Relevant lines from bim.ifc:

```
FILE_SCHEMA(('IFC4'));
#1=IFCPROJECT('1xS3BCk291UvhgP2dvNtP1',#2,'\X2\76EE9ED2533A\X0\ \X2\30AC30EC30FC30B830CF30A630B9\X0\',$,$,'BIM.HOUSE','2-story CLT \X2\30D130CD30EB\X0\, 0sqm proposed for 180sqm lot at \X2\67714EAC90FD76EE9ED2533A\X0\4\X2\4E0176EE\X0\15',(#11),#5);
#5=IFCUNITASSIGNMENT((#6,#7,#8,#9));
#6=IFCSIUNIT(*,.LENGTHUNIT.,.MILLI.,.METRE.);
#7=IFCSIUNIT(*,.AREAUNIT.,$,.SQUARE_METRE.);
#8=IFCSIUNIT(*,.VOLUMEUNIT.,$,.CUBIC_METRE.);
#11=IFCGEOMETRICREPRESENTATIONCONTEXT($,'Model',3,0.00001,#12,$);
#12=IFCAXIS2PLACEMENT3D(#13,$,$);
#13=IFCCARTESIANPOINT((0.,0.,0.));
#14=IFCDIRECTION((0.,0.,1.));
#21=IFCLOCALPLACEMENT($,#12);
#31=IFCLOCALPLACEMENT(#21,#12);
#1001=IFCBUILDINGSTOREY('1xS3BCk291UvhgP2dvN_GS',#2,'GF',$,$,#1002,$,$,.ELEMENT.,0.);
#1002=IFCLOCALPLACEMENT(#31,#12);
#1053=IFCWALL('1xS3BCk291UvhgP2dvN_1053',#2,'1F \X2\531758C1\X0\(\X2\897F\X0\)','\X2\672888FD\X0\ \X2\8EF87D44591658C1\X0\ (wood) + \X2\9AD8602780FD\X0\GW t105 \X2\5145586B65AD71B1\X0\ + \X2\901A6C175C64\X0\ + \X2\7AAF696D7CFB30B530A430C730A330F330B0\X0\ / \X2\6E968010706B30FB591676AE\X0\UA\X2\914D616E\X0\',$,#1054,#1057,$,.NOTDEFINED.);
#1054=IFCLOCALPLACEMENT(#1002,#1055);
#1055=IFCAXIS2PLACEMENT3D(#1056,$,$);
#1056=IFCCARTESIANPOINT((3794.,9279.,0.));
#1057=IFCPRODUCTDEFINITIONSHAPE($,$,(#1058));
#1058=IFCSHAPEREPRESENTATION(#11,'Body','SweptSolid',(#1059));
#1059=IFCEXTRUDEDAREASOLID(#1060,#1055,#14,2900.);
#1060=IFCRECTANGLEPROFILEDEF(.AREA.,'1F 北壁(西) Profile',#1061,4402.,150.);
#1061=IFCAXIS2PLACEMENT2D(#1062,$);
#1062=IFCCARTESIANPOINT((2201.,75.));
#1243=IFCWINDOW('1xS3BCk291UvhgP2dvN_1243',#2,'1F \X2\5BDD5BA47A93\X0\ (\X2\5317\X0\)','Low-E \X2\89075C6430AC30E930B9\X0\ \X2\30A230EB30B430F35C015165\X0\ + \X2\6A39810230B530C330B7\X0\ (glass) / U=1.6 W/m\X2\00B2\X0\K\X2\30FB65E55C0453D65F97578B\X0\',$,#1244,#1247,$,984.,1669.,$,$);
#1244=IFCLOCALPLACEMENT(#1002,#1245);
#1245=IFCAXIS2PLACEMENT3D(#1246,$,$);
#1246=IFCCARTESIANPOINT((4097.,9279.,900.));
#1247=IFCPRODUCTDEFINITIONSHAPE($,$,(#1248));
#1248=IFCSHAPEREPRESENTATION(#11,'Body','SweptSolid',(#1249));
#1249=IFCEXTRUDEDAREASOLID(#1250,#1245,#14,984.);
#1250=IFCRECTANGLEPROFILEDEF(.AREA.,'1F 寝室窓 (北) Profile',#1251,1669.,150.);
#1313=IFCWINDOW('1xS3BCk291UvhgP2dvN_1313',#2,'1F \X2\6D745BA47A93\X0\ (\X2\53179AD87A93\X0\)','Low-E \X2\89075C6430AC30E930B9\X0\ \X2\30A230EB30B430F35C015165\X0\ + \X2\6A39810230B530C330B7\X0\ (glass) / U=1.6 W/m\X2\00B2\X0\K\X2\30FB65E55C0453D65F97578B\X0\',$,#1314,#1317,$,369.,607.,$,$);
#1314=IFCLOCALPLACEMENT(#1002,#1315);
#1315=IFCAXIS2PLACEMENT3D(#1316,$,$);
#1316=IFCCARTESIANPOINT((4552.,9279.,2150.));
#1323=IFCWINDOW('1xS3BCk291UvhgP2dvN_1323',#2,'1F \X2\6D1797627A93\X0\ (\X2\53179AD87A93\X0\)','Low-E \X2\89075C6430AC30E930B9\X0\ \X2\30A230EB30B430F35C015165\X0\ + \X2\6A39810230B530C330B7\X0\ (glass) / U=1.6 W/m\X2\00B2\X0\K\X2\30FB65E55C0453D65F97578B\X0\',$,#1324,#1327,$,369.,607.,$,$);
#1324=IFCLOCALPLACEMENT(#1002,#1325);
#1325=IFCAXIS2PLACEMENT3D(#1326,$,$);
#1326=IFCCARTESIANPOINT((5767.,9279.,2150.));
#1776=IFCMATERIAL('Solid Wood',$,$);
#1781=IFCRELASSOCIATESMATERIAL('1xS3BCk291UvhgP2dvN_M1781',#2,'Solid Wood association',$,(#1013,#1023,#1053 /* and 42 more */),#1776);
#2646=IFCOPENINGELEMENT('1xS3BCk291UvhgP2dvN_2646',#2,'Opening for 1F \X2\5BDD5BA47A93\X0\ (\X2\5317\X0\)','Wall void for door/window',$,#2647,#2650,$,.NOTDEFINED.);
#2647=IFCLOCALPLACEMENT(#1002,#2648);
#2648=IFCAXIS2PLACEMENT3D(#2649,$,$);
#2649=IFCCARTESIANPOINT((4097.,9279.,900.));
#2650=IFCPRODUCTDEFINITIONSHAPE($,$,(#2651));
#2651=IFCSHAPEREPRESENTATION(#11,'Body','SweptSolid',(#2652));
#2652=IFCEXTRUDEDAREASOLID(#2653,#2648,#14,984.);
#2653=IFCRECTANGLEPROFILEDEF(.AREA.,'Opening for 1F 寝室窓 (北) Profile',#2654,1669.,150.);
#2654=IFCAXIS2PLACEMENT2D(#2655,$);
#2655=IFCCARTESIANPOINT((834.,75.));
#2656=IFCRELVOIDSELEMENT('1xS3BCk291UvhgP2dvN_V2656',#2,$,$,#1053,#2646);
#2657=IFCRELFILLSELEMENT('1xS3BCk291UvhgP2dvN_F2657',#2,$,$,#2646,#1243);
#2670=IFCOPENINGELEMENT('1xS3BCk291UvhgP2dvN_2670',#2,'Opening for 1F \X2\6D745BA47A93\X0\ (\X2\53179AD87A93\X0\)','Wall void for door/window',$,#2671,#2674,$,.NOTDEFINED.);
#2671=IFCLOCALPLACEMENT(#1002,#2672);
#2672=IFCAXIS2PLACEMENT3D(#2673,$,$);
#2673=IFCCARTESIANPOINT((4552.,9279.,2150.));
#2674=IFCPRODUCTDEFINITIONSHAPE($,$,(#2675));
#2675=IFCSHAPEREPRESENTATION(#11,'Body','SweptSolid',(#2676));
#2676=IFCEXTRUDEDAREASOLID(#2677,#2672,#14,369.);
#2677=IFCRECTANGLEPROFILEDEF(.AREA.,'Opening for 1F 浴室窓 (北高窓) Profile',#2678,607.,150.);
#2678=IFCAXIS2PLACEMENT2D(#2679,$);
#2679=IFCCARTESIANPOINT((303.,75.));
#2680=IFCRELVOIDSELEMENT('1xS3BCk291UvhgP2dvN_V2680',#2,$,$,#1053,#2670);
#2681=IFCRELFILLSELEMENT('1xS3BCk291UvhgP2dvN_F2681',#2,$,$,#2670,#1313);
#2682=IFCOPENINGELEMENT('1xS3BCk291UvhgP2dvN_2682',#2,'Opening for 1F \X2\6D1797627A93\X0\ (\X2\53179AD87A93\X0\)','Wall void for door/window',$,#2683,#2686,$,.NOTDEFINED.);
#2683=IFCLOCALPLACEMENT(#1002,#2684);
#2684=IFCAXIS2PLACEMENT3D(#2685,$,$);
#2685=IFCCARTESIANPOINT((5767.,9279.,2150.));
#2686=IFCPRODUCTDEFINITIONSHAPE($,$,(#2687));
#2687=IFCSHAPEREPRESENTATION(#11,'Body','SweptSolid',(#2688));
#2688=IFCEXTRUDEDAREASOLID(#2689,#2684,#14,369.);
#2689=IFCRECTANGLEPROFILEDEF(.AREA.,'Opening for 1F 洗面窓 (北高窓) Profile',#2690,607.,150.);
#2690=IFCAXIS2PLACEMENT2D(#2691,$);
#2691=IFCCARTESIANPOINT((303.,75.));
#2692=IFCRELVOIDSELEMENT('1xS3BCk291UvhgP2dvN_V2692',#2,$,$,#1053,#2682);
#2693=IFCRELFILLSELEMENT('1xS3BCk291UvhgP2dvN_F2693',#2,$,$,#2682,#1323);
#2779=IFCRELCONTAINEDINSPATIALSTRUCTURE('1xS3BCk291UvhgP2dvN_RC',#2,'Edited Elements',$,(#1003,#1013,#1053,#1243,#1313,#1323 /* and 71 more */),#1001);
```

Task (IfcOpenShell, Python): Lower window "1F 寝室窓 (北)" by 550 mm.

```python
import numpy as np
import ifcopenshell
import ifcopenshell.api.geometry
import ifcopenshell.util.placement
import ifcopenshell.util.unit

model = ifcopenshell.open("bim.ifc")
unit_scale = ifcopenshell.util.unit.calculate_unit_scale(model)

window = model.by_guid("1xS3BCk291UvhgP2dvN_1243")
opening = window.FillsVoids[0].RelatingOpeningElement
dz = -550.0

shift = np.array([0.0, 0.0, dz])
# The window is not placed relative to its opening, so move both.
for product in (opening, window):
    matrix = ifcopenshell.util.placement.get_local_placement(product.ObjectPlacement)
    matrix[:3, 3] += shift
    ifcopenshell.api.geometry.edit_object_placement(model, product=product, matrix=matrix, is_si=False)

print(f"moved by {dz * unit_scale:+.3f} m")

model.write("bim_updated.ifc")
```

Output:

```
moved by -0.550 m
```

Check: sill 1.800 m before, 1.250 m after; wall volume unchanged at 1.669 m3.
